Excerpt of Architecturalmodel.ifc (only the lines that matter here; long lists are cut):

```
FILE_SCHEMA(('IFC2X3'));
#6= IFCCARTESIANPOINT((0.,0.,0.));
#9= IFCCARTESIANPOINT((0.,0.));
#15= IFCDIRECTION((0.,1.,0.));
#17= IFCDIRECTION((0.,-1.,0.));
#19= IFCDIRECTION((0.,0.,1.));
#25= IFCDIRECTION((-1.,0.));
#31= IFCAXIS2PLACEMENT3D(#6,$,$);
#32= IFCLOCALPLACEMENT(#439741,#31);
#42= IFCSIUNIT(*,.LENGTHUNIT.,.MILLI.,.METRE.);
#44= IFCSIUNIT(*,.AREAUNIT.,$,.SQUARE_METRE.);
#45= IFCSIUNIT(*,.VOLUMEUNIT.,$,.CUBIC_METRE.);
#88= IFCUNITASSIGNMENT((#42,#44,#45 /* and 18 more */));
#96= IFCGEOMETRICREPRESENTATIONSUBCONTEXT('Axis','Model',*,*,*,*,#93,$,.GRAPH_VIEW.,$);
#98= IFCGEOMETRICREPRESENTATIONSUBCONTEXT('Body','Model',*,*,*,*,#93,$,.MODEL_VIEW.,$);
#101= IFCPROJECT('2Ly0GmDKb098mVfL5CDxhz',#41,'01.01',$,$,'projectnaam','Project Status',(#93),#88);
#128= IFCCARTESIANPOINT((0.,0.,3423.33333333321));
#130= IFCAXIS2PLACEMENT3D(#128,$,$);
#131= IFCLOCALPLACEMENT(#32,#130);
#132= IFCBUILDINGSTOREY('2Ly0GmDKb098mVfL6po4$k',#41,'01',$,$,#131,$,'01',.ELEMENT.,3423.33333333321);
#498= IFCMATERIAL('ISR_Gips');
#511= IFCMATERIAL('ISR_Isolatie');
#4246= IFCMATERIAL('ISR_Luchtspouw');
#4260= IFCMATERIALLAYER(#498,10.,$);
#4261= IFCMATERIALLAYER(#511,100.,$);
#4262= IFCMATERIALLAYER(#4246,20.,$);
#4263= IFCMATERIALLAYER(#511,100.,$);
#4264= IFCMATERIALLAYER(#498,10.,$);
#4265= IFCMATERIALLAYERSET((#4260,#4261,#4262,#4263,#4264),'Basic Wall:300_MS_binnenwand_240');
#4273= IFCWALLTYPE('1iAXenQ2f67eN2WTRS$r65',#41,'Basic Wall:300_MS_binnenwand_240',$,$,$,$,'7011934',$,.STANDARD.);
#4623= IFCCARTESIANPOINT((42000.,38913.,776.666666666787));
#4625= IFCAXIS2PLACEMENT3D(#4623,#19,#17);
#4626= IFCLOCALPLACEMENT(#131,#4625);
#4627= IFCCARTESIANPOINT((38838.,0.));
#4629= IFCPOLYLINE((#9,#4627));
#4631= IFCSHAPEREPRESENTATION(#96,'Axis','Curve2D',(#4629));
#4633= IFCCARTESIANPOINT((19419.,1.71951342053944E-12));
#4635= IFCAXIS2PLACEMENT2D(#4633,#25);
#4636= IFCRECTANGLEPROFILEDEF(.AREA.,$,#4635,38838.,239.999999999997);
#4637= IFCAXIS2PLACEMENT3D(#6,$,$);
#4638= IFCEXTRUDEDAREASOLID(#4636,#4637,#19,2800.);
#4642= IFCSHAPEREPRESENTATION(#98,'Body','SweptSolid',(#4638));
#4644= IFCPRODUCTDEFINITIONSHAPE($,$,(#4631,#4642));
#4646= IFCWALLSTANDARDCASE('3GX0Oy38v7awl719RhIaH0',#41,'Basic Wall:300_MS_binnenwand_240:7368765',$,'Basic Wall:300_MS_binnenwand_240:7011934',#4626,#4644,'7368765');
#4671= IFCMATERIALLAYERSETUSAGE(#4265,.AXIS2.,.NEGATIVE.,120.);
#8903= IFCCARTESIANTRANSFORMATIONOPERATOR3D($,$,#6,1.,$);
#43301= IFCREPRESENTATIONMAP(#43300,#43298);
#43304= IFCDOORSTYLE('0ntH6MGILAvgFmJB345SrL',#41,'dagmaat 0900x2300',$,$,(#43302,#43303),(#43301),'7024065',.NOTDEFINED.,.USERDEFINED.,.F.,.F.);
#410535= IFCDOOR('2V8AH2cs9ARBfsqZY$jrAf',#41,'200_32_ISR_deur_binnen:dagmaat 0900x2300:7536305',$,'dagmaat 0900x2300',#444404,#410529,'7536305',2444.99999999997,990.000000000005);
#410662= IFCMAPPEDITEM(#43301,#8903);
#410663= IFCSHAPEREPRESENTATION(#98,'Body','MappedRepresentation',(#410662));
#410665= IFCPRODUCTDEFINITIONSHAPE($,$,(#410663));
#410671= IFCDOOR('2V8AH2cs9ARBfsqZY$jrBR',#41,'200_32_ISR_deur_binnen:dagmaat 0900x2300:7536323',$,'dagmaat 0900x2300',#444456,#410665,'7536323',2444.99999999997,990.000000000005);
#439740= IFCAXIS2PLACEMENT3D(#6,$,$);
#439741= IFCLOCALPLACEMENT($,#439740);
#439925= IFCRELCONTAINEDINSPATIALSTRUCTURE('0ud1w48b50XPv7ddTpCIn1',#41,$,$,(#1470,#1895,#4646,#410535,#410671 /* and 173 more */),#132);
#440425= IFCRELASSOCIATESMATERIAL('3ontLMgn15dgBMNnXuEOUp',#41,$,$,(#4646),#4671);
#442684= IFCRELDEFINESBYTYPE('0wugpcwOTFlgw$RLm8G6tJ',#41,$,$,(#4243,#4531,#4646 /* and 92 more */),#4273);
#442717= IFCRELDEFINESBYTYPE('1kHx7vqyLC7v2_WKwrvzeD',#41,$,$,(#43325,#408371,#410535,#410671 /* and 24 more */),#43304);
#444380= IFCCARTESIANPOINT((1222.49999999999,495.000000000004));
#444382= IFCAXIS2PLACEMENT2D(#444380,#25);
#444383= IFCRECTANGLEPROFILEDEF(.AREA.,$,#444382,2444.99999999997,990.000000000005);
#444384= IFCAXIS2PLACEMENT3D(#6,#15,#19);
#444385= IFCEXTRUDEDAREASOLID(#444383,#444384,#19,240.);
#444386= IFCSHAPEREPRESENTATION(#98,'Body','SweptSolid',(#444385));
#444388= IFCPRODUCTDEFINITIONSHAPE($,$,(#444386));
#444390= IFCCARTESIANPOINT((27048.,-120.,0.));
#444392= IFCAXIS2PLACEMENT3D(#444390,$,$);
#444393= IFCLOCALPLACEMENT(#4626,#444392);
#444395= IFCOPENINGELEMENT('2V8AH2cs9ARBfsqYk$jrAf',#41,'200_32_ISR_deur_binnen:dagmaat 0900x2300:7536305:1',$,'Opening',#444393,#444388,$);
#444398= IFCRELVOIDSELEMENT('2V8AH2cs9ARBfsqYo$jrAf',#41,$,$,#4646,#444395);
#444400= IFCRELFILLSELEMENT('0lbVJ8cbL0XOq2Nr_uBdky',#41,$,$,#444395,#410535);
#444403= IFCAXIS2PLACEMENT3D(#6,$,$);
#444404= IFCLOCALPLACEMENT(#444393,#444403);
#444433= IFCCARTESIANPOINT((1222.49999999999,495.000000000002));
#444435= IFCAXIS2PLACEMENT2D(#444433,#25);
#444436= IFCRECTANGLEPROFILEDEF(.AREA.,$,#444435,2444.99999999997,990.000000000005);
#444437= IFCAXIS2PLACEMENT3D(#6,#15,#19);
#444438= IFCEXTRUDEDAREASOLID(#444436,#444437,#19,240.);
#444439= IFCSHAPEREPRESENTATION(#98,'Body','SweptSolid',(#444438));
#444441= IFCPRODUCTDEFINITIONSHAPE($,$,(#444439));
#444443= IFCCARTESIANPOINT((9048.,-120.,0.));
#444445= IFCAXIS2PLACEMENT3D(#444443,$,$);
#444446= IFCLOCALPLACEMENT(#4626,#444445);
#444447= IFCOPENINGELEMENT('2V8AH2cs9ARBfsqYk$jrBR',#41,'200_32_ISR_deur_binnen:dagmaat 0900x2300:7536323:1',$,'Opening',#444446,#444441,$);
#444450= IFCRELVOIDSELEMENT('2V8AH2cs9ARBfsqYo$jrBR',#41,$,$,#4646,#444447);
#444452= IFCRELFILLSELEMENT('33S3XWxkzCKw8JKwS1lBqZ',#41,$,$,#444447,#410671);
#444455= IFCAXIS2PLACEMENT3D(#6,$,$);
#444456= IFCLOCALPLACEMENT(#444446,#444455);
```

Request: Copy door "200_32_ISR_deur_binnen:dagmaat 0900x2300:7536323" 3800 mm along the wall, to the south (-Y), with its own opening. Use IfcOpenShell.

```python
import ifcopenshell
import ifcopenshell.api.feature
import ifcopenshell.api.geometry
import ifcopenshell.api.root
import ifcopenshell.geom
import ifcopenshell.util.element
import ifcopenshell.util.placement
import ifcopenshell.util.shape

model = ifcopenshell.open("Architecturalmodel.ifc")
settings = ifcopenshell.geom.settings()


def volume(element):
    """Net volume in cubic metres, openings subtracted."""
    shape = ifcopenshell.geom.create_shape(settings, element)
    return ifcopenshell.util.shape.get_volume(shape.geometry)


def reuse_history(source, copy):
    """copy_class also copies each property set's owner history, people and application; keep the originals."""
    for rel in copy.IsDefinedBy:
        if rel.is_a("IfcRelDefinesByProperties") and (history := rel.RelatingPropertyDefinition.OwnerHistory):
            rel.RelatingPropertyDefinition.OwnerHistory = source.OwnerHistory
            ifcopenshell.util.element.remove_deep2(model, history)


door = model.by_guid("2V8AH2cs9ARBfsqZY$jrBR")
opening = door.FillsVoids[0].RelatingOpeningElement
wall = opening.VoidsElements[0].RelatingBuildingElement
before = volume(wall)
shift = ifcopenshell.util.placement.get_local_placement(wall.ObjectPlacement)[:3, 0] * 3800.0

# copy_class copies the void relationship, type, container and properties, but no geometry.
new_opening = ifcopenshell.api.root.copy_class(model, product=opening)
new_opening.Representation = ifcopenshell.util.element.copy_deep(
    model, opening.Representation, exclude=["IfcGeometricRepresentationContext", "IfcRepresentationMap"]
)
new_opening.Name = "200_32_ISR_deur_binnen:dagmaat 0900x2300"
new_door = ifcopenshell.api.root.copy_class(model, product=door)
new_door.Representation = ifcopenshell.util.element.copy_deep(
    model, door.Representation, exclude=["IfcGeometricRepresentationContext", "IfcRepresentationMap"]
)
new_door.Name = "200_32_ISR_deur_binnen:dagmaat 0900x2300"
new_door.Tag = None
reuse_history(door, new_door)
fills = ifcopenshell.api.feature.add_filling(model, opening=new_opening, element=new_door)
fills.OwnerHistory = new_door.OwnerHistory  # required in IFC2X3

for old, new in ((opening, new_opening), (door, new_door)):
    matrix = ifcopenshell.util.placement.get_local_placement(old.ObjectPlacement)
    matrix[:3, 3] += shift
    ifcopenshell.api.geometry.edit_object_placement(model, product=new, matrix=matrix, is_si=False)

after = volume(wall)

print(f"wall volume {before:.3f} -> {after:.3f} m3")

model.write("Architecturalmodel_rev.ifc")
```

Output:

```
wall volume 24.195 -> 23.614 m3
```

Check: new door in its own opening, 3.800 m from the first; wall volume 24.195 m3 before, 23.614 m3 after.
